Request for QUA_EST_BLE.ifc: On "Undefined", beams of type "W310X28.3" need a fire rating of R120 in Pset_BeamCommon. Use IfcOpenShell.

First a look at what the model holds.

```python
import ifcopenshell
import ifcopenshell.util.element

model = ifcopenshell.open("QUA_EST_BLE.ifc")
print(model.schema)
storey = next(s for s in model.by_type("IfcBuildingStorey") if s.Name == "Undefined")
beams = [e for e in ifcopenshell.util.element.get_decomposition(storey) if e.is_a("IfcBeam")]
seen = {}
for e in beams:
    element_type = ifcopenshell.util.element.get_type(e)
    key = (element_type.Name if element_type != e and element_type else None, ifcopenshell.util.element.get_pset(e, "Pset_BeamCommon", "FireRating"))
    seen[key] = seen.get(key, 0) + 1
for (name, value), count in sorted(seen.items(), key=str):
    print(count, "x", name, "|", value)
```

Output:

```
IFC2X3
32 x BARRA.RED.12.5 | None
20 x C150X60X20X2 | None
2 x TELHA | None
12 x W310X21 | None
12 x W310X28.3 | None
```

```python
import ifcopenshell
import ifcopenshell.api.pset
import ifcopenshell.util.element

model = ifcopenshell.open("QUA_EST_BLE.ifc")

storey = next(s for s in model.by_type("IfcBuildingStorey") if s.Name == "Undefined")
beams = [e for e in ifcopenshell.util.element.get_decomposition(storey) if e.is_a("IfcBeam")]

count = 0
for e in beams:
    element_type = ifcopenshell.util.element.get_type(e)
    if element_type in (None, e) or element_type.Name != "W310X28.3":
        continue
    found = ifcopenshell.util.element.get_pset(e, "Pset_BeamCommon", should_inherit=False)
    if found:
        pset = model.by_id(found["id"])
        if len(ifcopenshell.util.element.get_elements_by_pset(pset)) > 1:
            pset = ifcopenshell.api.pset.unshare_pset(model, products=[e], pset=pset)[0]
    else:
        pset = ifcopenshell.api.pset.add_pset(model, product=e, name="Pset_BeamCommon")
    ifcopenshell.api.pset.edit_pset(model, pset=pset, properties={"FireRating": "R120"})
    count += 1

print(count, "beams updated")

model.write("QUA_EST_BLE_rev.ifc")
```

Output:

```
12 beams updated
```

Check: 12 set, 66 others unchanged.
